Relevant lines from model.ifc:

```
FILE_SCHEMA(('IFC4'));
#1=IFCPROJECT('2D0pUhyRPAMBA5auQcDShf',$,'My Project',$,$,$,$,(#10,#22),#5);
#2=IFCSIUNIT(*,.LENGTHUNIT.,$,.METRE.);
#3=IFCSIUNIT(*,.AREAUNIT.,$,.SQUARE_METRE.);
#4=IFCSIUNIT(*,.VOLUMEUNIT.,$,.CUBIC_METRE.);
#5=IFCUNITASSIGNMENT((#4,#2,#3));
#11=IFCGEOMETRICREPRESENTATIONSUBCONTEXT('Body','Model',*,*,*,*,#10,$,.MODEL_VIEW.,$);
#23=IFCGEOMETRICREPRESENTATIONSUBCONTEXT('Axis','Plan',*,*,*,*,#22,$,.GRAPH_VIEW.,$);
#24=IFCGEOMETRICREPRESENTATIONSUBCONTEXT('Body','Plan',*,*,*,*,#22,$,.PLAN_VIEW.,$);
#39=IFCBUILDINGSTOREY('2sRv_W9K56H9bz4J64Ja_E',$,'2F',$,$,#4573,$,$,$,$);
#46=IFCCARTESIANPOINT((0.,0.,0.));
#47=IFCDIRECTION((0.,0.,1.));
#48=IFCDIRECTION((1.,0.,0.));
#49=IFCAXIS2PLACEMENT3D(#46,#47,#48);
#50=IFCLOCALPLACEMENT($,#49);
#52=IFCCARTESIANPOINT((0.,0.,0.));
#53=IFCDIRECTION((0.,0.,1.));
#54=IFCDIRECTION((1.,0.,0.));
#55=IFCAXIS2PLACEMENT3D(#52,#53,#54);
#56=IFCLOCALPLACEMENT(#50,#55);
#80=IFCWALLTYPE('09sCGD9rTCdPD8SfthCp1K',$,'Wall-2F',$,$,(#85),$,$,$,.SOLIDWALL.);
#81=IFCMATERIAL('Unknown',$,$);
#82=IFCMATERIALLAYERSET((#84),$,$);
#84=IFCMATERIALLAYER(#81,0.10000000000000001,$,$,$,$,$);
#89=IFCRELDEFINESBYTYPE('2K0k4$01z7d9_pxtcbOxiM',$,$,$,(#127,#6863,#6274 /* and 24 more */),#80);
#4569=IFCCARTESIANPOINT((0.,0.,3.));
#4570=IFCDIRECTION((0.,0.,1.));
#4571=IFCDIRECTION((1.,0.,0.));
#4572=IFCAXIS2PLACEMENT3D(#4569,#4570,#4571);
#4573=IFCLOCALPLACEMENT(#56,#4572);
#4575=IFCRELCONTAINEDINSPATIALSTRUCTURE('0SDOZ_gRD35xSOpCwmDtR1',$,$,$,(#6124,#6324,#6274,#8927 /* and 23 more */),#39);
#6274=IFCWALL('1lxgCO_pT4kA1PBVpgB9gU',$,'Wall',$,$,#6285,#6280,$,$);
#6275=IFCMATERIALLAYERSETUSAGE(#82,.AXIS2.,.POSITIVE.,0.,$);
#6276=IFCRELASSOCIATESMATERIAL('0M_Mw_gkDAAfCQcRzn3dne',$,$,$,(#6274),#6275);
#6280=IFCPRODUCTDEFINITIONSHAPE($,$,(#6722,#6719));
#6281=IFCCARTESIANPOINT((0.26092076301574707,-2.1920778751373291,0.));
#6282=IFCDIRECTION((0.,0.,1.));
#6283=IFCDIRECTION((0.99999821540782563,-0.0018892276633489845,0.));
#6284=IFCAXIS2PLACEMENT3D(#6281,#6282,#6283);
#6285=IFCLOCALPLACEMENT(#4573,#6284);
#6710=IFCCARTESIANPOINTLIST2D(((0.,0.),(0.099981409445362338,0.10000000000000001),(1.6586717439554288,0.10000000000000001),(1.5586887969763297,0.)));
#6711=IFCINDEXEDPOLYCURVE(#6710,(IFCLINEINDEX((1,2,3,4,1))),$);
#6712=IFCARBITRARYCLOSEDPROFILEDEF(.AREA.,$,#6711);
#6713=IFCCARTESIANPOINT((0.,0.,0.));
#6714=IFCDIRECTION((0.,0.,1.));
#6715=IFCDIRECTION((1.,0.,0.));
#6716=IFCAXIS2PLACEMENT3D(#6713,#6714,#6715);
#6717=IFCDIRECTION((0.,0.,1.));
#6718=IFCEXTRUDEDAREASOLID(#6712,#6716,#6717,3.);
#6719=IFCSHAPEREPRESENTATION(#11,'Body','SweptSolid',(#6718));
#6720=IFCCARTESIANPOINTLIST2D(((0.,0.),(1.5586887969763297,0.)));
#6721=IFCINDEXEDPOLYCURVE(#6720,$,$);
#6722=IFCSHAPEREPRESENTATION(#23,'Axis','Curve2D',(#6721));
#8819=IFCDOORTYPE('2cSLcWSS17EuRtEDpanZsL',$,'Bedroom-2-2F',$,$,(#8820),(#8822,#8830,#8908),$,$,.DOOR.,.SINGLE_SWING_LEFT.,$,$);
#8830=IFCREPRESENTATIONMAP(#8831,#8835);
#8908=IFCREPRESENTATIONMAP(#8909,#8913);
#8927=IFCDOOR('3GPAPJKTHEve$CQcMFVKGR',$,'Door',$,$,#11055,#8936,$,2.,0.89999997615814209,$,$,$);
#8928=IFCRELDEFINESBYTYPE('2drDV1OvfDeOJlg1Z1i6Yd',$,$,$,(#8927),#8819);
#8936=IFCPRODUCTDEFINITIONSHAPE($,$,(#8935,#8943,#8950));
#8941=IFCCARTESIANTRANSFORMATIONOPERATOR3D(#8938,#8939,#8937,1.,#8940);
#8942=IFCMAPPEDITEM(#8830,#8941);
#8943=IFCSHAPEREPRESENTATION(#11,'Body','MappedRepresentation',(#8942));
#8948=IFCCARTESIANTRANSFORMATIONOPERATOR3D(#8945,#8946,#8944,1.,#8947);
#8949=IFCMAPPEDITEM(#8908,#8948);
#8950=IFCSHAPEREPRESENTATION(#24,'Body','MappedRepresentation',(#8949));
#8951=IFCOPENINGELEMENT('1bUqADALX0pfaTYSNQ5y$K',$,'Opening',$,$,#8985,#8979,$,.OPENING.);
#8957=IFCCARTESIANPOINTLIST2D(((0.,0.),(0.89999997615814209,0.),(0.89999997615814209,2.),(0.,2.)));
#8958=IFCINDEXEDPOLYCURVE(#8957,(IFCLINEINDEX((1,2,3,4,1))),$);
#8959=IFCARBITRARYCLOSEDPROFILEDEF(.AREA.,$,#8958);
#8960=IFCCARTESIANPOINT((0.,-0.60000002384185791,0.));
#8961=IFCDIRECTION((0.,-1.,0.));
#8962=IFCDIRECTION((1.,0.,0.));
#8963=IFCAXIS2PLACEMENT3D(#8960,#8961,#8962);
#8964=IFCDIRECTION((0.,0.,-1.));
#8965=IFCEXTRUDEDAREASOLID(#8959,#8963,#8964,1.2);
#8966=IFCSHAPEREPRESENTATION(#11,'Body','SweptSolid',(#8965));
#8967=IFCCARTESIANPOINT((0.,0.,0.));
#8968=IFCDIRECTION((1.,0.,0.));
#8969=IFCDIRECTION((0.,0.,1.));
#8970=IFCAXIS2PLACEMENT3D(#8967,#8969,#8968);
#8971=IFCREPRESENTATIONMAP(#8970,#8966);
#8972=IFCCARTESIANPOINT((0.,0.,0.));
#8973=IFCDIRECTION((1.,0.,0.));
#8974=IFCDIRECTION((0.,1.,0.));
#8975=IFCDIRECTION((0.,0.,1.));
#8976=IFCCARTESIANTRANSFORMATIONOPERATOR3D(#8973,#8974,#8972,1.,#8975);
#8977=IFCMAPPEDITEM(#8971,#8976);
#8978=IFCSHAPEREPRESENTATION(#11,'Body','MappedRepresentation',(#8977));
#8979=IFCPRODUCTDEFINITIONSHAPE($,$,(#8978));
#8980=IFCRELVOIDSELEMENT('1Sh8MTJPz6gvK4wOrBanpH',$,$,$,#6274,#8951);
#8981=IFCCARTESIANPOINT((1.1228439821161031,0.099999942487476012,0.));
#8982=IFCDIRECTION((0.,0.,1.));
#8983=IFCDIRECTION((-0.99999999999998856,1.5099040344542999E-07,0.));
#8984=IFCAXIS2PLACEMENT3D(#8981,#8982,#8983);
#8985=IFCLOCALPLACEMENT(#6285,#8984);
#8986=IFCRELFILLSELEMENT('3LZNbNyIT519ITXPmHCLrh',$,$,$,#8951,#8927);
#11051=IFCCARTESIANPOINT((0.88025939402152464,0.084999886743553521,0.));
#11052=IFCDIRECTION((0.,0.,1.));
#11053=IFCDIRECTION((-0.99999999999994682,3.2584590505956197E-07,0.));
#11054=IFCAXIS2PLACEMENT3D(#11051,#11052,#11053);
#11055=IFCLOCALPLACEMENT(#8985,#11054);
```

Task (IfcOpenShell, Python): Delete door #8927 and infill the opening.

```python
import ifcopenshell
import ifcopenshell.api.feature
import ifcopenshell.api.root
import ifcopenshell.geom
import ifcopenshell.util.shape

model = ifcopenshell.open("model.ifc")
settings = ifcopenshell.geom.settings()


def volume(element):
    """Net volume in cubic metres, openings subtracted."""
    shape = ifcopenshell.geom.create_shape(settings, element)
    return ifcopenshell.util.shape.get_volume(shape.geometry)


door = model.by_guid("3GPAPJKTHEve$CQcMFVKGR")
opening = door.FillsVoids[0].RelatingOpeningElement
wall = opening.VoidsElements[0].RelatingBuildingElement
before = volume(wall)

ifcopenshell.api.root.remove_product(model, product=door)
ifcopenshell.api.feature.remove_feature(model, feature=opening)

after = volume(wall)

print(f"wall volume {before:.3f} -> {after:.3f} m3")

model.write("model_rev.ifc")
```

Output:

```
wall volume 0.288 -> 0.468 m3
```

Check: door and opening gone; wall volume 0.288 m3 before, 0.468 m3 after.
